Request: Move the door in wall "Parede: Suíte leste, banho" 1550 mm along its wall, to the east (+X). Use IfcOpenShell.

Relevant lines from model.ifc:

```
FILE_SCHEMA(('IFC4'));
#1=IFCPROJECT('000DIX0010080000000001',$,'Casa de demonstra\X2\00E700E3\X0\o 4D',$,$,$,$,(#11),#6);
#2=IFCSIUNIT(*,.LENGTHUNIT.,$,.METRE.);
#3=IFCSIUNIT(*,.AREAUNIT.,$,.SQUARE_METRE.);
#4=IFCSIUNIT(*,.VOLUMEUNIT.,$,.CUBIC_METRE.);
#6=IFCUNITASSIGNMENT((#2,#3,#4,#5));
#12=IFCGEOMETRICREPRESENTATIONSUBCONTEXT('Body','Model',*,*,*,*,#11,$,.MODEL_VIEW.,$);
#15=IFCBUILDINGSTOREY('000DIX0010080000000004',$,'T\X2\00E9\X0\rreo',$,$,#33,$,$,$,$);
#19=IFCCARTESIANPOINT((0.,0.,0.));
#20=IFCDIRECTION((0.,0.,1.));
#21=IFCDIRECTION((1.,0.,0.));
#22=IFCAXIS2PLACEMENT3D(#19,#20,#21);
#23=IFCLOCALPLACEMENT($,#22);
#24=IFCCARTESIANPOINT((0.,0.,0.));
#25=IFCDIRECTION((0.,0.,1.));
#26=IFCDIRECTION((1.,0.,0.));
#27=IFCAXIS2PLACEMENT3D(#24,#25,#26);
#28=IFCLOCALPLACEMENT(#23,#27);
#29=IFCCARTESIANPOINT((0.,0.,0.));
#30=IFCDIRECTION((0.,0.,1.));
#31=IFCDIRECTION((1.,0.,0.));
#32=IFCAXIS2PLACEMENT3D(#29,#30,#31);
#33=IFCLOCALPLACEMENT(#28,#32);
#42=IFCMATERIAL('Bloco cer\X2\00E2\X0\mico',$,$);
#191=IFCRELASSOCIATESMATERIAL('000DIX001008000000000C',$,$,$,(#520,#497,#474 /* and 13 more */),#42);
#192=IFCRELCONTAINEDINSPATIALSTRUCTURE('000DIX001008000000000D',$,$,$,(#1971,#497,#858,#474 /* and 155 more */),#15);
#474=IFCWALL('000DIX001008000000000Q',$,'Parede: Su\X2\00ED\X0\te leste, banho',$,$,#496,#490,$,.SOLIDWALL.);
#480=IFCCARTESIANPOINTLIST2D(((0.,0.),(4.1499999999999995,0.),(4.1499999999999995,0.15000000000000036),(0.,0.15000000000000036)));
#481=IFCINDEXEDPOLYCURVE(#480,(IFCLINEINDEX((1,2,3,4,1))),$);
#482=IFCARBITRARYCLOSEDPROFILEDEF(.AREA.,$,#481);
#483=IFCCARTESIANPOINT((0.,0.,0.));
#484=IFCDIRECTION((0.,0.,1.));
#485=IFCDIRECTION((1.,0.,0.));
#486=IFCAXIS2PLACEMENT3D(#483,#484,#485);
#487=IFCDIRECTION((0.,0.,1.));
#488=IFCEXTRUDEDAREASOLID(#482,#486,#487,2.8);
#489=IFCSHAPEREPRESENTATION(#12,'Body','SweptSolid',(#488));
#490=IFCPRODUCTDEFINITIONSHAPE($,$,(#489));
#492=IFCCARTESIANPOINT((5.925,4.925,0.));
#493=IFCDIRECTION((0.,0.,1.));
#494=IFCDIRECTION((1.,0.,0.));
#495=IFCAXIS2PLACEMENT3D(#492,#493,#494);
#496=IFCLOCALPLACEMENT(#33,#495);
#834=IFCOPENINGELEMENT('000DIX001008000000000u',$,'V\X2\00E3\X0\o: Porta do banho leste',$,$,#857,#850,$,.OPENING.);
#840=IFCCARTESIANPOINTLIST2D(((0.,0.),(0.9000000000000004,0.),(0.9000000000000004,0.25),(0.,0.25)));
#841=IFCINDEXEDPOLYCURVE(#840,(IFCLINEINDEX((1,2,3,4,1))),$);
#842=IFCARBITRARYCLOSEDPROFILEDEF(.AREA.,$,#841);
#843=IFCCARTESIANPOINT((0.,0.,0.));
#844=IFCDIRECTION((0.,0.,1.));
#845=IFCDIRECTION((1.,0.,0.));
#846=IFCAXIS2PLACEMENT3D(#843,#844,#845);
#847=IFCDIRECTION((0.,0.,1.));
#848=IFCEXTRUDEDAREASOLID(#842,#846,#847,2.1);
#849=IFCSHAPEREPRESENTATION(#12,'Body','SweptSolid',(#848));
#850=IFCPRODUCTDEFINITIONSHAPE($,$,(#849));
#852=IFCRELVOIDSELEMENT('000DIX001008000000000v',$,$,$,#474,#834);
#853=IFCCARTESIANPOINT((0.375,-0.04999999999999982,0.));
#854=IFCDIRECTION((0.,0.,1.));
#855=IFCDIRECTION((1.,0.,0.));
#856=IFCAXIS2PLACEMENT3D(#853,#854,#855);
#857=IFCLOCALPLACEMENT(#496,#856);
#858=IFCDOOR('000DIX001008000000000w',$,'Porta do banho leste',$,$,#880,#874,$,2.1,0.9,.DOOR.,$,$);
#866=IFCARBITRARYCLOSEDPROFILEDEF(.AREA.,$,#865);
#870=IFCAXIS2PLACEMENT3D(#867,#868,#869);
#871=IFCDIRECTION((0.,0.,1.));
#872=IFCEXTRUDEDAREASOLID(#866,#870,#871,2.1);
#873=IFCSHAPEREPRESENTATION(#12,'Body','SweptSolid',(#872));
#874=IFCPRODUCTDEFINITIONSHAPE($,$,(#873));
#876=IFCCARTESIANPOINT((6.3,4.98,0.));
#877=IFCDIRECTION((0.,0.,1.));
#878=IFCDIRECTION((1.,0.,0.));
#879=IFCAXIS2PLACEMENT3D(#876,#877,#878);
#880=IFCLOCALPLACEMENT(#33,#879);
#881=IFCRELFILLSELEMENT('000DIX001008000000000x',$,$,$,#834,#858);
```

```python
import ifcopenshell
import ifcopenshell.api.geometry
import ifcopenshell.util.placement
import ifcopenshell.util.unit

model = ifcopenshell.open("model.ifc")
unit_scale = ifcopenshell.util.unit.calculate_unit_scale(model)

door = model.by_guid("000DIX001008000000000w")
opening = door.FillsVoids[0].RelatingOpeningElement
wall = opening.VoidsElements[0].RelatingBuildingElement

wall_matrix = ifcopenshell.util.placement.get_local_placement(wall.ObjectPlacement)
shift = wall_matrix[:3, 0] * 1.55 / unit_scale
before = ifcopenshell.util.placement.get_local_placement(door.ObjectPlacement)[:3, 3].copy()

# The door is not placed relative to its opening, so move both.
for product in (opening, door):
    matrix = ifcopenshell.util.placement.get_local_placement(product.ObjectPlacement)
    matrix[:3, 3] += shift
    ifcopenshell.api.geometry.edit_object_placement(model, product=product, matrix=matrix, is_si=False)

after = ifcopenshell.util.placement.get_local_placement(door.ObjectPlacement)[:3, 3]
print("door moved by", (after - before).round(3) + 0.0)

model.write("model_edited.ifc")
```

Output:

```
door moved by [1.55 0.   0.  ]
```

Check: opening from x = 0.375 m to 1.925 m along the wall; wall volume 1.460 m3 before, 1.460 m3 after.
